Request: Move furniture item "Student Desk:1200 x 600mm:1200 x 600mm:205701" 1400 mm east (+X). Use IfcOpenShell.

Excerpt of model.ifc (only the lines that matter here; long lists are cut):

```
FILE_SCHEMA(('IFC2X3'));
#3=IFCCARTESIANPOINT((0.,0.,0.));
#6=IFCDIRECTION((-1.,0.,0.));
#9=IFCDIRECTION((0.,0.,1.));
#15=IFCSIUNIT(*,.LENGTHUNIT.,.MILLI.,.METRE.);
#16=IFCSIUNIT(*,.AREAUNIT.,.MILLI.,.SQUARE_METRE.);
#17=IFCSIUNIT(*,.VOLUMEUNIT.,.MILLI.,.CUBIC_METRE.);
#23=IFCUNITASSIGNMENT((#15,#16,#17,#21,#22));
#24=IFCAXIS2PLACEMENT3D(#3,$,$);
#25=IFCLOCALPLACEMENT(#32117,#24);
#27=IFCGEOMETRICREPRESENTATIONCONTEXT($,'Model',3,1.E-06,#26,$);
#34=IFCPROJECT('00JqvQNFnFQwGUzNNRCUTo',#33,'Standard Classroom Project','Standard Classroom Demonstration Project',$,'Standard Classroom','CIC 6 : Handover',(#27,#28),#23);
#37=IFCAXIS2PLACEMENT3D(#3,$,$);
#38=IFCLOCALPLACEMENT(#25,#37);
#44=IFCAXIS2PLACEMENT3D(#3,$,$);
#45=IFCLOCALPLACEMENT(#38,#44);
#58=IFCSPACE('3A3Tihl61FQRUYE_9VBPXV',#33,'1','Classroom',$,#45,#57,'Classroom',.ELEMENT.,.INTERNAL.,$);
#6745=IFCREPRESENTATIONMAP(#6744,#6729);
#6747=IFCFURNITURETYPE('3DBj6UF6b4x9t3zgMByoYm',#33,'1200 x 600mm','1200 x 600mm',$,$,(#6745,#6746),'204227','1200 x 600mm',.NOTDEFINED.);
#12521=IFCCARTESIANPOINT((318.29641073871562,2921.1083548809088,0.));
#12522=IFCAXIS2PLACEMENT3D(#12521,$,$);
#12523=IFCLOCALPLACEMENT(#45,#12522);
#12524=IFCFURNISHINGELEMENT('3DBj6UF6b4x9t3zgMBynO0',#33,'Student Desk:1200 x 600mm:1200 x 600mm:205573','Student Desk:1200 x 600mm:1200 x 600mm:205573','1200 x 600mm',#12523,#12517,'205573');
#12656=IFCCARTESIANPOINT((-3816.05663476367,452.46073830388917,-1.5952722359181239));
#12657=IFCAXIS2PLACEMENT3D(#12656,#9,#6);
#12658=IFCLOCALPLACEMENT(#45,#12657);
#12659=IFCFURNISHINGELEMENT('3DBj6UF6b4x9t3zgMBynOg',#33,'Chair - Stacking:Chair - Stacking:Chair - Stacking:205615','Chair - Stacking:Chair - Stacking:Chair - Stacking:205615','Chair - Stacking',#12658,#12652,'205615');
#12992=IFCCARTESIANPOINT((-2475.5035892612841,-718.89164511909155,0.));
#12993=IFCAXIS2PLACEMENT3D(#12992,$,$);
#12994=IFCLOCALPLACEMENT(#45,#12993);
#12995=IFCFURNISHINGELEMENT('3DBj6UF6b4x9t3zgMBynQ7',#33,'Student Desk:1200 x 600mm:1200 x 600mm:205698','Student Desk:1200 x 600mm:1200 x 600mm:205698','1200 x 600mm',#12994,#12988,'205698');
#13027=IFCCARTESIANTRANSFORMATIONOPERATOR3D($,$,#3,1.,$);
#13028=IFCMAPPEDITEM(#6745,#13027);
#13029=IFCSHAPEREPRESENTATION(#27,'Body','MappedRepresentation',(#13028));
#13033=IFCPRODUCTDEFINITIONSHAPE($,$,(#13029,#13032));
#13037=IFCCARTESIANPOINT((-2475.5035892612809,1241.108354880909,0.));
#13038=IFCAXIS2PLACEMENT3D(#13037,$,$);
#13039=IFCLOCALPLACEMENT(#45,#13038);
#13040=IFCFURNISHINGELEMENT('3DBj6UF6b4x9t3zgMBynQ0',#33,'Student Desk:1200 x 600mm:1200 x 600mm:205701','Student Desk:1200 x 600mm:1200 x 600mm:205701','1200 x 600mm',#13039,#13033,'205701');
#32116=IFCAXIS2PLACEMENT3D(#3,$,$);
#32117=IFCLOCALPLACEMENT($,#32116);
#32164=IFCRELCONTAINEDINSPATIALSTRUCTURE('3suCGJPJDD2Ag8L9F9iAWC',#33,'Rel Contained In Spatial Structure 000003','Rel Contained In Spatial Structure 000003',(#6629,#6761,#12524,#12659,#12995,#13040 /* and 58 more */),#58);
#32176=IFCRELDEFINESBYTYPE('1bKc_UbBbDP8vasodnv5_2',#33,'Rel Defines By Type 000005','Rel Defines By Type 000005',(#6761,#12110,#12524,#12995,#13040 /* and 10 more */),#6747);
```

```python
import ifcopenshell
import ifcopenshell.api.geometry
import ifcopenshell.util.placement
import ifcopenshell.util.unit

model = ifcopenshell.open("model.ifc")
unit_scale = ifcopenshell.util.unit.calculate_unit_scale(model)

item = model.by_guid("3DBj6UF6b4x9t3zgMBynQ0")
matrix = ifcopenshell.util.placement.get_local_placement(item.ObjectPlacement)
matrix[0, 3] += 1.4 / unit_scale
ifcopenshell.api.geometry.edit_object_placement(model, product=item, matrix=matrix, is_si=False)

print(ifcopenshell.util.placement.get_local_placement(item.ObjectPlacement).round(3) + 0.0)

model.write("model-out.ifc")
```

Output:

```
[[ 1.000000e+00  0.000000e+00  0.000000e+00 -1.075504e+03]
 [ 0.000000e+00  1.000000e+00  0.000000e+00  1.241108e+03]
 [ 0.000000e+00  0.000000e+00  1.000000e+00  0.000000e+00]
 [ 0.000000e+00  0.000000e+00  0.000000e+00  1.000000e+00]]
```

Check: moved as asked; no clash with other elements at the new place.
